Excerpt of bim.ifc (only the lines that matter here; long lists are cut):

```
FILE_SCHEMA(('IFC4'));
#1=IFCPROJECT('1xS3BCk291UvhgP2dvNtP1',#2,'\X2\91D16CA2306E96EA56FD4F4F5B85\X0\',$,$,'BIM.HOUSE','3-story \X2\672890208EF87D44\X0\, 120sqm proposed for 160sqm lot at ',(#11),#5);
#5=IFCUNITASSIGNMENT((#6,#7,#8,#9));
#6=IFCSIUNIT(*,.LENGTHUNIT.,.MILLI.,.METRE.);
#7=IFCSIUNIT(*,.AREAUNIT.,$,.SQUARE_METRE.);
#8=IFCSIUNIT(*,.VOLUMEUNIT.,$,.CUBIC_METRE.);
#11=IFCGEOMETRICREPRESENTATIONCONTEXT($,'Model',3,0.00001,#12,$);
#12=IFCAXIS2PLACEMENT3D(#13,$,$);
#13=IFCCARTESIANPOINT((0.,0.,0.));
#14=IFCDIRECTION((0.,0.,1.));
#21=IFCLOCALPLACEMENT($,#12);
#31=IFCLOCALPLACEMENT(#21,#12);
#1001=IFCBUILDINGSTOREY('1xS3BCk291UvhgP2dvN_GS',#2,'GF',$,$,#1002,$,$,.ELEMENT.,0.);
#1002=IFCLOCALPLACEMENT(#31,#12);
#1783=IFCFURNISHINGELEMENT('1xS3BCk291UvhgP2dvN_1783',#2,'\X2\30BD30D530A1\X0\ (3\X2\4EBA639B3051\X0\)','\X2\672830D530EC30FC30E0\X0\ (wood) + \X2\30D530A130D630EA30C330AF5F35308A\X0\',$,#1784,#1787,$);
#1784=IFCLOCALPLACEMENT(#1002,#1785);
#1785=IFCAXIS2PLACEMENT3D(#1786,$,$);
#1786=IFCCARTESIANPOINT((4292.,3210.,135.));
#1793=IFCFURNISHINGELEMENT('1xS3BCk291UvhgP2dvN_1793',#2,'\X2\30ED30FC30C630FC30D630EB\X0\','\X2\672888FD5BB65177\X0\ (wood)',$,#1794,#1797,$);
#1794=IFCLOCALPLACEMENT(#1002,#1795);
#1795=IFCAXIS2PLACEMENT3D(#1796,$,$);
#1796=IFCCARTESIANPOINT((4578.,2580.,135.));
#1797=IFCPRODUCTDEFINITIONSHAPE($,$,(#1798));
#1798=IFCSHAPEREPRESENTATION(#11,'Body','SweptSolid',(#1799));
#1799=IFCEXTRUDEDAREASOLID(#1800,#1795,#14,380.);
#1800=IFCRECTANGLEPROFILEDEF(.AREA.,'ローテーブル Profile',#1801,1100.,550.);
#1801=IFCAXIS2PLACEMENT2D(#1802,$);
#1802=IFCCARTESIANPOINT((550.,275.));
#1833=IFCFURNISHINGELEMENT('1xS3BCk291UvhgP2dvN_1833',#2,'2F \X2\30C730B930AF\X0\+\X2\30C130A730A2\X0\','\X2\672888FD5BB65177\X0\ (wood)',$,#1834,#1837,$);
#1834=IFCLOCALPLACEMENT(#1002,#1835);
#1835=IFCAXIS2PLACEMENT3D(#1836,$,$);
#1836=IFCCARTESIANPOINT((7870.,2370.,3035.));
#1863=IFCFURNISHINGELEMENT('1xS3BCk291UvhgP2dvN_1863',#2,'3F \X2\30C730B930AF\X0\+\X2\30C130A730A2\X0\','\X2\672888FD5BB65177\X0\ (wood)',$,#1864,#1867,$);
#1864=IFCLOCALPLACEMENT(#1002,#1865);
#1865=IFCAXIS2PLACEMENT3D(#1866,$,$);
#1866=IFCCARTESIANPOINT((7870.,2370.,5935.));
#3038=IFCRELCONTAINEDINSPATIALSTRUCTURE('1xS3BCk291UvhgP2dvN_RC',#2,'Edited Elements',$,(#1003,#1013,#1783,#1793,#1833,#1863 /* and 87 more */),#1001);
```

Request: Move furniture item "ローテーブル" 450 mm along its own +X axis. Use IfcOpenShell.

```python
import ifcopenshell
import ifcopenshell.api.geometry
import ifcopenshell.util.placement
import ifcopenshell.util.unit

model = ifcopenshell.open("bim.ifc")
unit_scale = ifcopenshell.util.unit.calculate_unit_scale(model)

item = model.by_id(1793)
matrix = ifcopenshell.util.placement.get_local_placement(item.ObjectPlacement)
matrix[:3, 3] += matrix[:3, 0] * 0.45 / unit_scale
ifcopenshell.api.geometry.edit_object_placement(model, product=item, matrix=matrix, is_si=False)

print(ifcopenshell.util.placement.get_local_placement(item.ObjectPlacement).round(3) + 0.0)

model.write("bim_rev.ifc")
```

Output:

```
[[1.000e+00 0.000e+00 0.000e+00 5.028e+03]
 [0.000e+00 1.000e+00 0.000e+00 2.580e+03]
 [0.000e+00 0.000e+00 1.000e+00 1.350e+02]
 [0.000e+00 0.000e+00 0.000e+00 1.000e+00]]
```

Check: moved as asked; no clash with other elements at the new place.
